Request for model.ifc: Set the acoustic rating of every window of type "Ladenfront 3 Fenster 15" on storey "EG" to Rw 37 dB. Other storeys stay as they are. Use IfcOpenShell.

First a look at what the model holds.

```python
import ifcopenshell
import ifcopenshell.util.element

model = ifcopenshell.open("model.ifc")
print(model.schema)
storey = next(s for s in model.by_type("IfcBuildingStorey") if s.Name == "EG")
windows = [e for e in ifcopenshell.util.element.get_decomposition(storey) if e.is_a("IfcWindow")]
seen = {}
for e in windows:
    element_type = ifcopenshell.util.element.get_type(e)
    key = (element_type.Name if element_type != e and element_type else None, ifcopenshell.util.element.get_pset(e, "Pset_WindowCommon", "AcousticRating"))
    seen[key] = seen.get(key, 0) + 1
for (name, value), count in sorted(seen.items(), key=str):
    print(count, "x", name, "|", value)
```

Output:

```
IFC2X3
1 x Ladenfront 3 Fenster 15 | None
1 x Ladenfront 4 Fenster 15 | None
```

```python
import ifcopenshell
import ifcopenshell.api.pset
import ifcopenshell.util.element

model = ifcopenshell.open("model.ifc")

storey = next(s for s in model.by_type("IfcBuildingStorey") if s.Name == "EG")
windows = [e for e in ifcopenshell.util.element.get_decomposition(storey) if e.is_a("IfcWindow")]

count = 0
for e in windows:
    element_type = ifcopenshell.util.element.get_type(e)
    if element_type in (None, e) or element_type.Name != "Ladenfront 3 Fenster 15":
        continue
    # add_pset returns the element's existing set when there is one.
    pset = ifcopenshell.api.pset.add_pset(model, product=e, name="Pset_WindowCommon")
    ifcopenshell.api.pset.edit_pset(model, pset=pset, properties={"AcousticRating": "Rw 37 dB"})
    count += 1

print(count, "windows updated")

model.write("model_rev.ifc")
```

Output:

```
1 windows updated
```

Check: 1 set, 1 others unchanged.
